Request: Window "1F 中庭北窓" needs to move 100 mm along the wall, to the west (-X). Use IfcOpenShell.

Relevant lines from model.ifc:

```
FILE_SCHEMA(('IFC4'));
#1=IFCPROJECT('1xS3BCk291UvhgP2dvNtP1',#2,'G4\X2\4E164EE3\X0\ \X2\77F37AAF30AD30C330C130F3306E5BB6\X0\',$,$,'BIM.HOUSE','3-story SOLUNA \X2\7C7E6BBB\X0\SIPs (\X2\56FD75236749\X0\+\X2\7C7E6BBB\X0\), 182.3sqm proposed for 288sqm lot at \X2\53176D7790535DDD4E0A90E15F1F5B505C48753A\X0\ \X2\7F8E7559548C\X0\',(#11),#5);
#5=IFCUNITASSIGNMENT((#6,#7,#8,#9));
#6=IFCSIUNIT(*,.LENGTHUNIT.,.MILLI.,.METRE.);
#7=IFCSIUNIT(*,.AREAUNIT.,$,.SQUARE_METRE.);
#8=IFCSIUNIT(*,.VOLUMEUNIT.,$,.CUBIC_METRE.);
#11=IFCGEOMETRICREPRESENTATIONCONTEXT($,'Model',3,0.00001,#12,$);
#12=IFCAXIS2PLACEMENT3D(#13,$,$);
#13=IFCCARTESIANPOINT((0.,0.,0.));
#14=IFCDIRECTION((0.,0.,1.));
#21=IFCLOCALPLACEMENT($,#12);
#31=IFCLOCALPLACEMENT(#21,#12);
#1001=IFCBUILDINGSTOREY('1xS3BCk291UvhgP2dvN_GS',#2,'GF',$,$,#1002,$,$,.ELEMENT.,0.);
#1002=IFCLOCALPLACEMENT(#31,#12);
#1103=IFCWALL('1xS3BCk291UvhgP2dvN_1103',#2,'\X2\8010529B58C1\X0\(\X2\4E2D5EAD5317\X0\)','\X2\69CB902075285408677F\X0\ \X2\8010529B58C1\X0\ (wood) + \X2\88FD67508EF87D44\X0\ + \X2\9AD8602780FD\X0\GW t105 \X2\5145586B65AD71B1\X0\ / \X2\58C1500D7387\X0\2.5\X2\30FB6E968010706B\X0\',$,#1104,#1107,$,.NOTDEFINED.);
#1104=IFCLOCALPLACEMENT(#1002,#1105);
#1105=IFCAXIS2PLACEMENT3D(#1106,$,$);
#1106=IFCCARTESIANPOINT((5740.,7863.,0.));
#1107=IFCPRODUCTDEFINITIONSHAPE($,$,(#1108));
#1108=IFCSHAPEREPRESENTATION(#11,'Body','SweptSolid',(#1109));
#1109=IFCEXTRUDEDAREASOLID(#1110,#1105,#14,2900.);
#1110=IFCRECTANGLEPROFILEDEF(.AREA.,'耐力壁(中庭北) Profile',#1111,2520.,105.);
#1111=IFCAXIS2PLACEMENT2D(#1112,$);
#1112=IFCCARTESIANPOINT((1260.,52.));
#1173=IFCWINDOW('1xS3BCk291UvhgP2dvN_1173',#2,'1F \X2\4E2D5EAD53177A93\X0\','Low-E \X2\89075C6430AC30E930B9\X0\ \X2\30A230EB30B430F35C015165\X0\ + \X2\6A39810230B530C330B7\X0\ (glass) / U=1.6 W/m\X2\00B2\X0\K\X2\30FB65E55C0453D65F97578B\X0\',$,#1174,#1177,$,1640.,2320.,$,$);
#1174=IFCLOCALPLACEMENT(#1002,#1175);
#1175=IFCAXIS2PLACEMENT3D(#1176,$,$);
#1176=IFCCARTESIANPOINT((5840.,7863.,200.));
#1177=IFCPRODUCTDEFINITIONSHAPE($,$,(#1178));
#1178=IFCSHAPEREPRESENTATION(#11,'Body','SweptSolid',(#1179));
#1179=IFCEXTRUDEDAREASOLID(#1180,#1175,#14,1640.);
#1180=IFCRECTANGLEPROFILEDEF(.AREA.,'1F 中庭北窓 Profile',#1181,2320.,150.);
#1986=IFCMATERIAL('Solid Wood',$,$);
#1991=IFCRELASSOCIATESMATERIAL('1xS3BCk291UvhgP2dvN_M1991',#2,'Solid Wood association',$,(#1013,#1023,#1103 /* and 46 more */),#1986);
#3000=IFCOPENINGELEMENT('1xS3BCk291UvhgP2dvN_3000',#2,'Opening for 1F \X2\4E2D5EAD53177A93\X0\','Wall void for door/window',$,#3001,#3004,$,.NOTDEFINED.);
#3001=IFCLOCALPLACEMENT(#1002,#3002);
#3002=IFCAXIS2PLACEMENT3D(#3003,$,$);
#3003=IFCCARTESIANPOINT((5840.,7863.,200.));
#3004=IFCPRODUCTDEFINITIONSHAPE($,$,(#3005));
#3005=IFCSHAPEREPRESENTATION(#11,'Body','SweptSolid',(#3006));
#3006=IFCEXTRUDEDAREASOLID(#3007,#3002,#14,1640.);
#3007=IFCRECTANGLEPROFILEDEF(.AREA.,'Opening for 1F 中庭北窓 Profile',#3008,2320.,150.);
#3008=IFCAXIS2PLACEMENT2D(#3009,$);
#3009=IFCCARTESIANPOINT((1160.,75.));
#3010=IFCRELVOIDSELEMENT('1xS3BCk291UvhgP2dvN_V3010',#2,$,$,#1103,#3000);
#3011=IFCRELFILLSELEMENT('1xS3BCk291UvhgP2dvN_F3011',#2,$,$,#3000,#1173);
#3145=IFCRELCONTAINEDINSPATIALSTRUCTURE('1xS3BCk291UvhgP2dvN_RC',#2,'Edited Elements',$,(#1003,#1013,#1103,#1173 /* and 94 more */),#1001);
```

```python
import ifcopenshell
import ifcopenshell.api.geometry
import ifcopenshell.util.placement
import ifcopenshell.util.unit

model = ifcopenshell.open("model.ifc")
unit_scale = ifcopenshell.util.unit.calculate_unit_scale(model)

window = model.by_id(1173)
opening = window.FillsVoids[0].RelatingOpeningElement
wall = opening.VoidsElements[0].RelatingBuildingElement

wall_matrix = ifcopenshell.util.placement.get_local_placement(wall.ObjectPlacement)
shift = wall_matrix[:3, 0] * -0.1 / unit_scale
before = ifcopenshell.util.placement.get_local_placement(window.ObjectPlacement)[:3, 3].copy()

# The window is not placed relative to its opening, so move both.
for product in (opening, window):
    matrix = ifcopenshell.util.placement.get_local_placement(product.ObjectPlacement)
    matrix[:3, 3] += shift
    ifcopenshell.api.geometry.edit_object_placement(model, product=product, matrix=matrix, is_si=False)

after = ifcopenshell.util.placement.get_local_placement(window.ObjectPlacement)[:3, 3]
print("window moved by", (after - before).round(3) + 0.0)

model.write("model_v2.ifc")
```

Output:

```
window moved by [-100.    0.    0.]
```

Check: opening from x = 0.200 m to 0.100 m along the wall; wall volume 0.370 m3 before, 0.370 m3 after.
